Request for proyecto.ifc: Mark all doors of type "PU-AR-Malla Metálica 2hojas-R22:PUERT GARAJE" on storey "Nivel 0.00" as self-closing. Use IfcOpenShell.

First a look at what the model holds.

```python
import ifcopenshell
import ifcopenshell.util.element

model = ifcopenshell.open("proyecto.ifc")
print(model.schema)
storey = next(s for s in model.by_type("IfcBuildingStorey") if s.Name == "Nivel 0.00")
doors = [e for e in ifcopenshell.util.element.get_decomposition(storey) if e.is_a("IfcDoor")]
seen = {}
for e in doors:
    element_type = ifcopenshell.util.element.get_type(e)
    key = (element_type.Name if element_type != e and element_type else None, ifcopenshell.util.element.get_pset(e, "Pset_DoorCommon", "SelfClosing"))
    seen[key] = seen.get(key, 0) + 1
for (name, value), count in sorted(seen.items(), key=str):
    print(count, "x", name, "|", value)
```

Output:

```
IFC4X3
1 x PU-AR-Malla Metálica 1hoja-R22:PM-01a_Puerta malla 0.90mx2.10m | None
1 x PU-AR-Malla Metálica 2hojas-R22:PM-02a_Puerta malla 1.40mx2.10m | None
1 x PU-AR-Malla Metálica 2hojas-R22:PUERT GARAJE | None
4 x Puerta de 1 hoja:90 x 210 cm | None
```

```python
import ifcopenshell
import ifcopenshell.api.pset
import ifcopenshell.util.element

model = ifcopenshell.open("proyecto.ifc")

storey = next(s for s in model.by_type("IfcBuildingStorey") if s.Name == "Nivel 0.00")
doors = [e for e in ifcopenshell.util.element.get_decomposition(storey) if e.is_a("IfcDoor")]

count = 0
for e in doors:
    element_type = ifcopenshell.util.element.get_type(e)
    if element_type in (None, e) or element_type.Name != "PU-AR-Malla Metálica 2hojas-R22:PUERT GARAJE":
        continue
    # add_pset returns the element's existing set when there is one.
    pset = ifcopenshell.api.pset.add_pset(model, product=e, name="Pset_DoorCommon")
    ifcopenshell.api.pset.edit_pset(model, pset=pset, properties={"SelfClosing": True})
    count += 1

print(count, "doors updated")

model.write("proyecto_updated.ifc")
```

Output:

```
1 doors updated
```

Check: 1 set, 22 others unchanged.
